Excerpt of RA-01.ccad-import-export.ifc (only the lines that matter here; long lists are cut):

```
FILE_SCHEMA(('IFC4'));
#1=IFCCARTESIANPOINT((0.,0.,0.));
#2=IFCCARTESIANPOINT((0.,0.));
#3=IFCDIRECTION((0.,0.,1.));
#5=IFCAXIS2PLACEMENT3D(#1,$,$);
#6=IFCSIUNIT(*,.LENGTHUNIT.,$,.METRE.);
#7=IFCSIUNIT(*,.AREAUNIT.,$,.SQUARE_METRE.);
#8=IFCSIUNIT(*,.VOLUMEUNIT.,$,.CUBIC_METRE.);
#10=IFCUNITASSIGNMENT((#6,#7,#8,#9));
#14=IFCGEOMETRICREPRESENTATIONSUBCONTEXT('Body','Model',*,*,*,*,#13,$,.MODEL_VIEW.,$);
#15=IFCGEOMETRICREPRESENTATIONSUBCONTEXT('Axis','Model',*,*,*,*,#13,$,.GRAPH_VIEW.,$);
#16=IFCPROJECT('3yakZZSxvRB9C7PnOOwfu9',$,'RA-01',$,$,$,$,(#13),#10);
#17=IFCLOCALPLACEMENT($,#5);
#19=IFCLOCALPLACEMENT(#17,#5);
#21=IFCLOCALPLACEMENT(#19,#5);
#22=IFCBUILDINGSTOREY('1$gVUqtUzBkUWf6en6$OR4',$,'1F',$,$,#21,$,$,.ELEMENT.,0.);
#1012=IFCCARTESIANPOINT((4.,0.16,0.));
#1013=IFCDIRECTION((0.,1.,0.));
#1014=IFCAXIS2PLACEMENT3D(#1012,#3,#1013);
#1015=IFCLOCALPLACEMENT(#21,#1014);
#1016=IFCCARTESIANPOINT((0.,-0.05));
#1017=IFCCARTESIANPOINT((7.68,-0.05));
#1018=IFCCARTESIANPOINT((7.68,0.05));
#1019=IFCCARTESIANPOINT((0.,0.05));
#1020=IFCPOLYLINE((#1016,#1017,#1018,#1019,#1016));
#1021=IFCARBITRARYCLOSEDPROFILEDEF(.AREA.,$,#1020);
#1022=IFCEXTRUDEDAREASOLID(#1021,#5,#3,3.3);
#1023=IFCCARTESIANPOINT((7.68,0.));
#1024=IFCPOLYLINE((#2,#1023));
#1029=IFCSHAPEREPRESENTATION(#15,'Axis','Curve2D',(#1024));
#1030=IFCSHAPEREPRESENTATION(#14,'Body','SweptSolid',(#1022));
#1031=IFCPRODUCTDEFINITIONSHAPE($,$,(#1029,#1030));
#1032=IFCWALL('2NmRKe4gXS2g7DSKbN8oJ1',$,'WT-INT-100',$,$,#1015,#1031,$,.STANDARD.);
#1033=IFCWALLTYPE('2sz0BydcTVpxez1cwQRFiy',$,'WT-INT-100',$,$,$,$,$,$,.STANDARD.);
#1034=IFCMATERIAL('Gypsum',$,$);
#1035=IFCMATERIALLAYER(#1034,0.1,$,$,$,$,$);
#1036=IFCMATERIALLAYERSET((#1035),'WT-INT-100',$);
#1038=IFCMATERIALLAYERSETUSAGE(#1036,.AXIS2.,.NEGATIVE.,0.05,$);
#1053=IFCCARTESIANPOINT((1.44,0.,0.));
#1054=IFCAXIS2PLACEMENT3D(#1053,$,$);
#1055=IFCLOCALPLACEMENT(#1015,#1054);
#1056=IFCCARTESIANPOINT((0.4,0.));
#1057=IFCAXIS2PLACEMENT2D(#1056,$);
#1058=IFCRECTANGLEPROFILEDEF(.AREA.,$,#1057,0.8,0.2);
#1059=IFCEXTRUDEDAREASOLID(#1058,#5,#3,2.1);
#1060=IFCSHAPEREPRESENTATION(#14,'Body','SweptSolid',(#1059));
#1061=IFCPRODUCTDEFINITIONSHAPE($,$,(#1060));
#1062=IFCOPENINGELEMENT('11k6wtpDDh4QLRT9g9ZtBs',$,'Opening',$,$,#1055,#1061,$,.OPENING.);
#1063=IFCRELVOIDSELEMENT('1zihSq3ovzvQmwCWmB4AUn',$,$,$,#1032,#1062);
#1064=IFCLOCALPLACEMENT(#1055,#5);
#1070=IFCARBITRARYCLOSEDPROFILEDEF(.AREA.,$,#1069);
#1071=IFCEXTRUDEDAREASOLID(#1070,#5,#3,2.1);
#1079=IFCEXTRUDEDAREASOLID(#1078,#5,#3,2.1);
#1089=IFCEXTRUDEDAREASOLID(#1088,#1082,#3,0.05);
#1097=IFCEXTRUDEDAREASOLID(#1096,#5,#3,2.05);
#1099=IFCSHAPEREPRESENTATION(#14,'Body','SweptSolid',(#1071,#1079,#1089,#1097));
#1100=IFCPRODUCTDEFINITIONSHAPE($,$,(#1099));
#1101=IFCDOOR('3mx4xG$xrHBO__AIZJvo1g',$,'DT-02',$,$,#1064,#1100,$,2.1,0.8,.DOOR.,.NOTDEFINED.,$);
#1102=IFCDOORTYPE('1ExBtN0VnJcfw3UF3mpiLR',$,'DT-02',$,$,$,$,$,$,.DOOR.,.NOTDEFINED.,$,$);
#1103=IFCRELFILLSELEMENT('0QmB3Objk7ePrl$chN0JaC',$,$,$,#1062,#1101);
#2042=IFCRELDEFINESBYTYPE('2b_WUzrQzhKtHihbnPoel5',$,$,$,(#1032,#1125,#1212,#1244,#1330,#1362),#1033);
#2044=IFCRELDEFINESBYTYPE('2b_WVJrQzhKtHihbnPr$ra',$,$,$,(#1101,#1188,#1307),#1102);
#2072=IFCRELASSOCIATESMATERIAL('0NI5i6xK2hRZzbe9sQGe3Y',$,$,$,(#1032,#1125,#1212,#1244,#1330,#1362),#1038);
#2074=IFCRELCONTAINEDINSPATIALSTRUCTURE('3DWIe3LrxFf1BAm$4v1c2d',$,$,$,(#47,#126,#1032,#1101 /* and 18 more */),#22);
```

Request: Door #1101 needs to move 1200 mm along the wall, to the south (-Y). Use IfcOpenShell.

```python
import ifcopenshell
import ifcopenshell.api.geometry
import ifcopenshell.util.placement
import ifcopenshell.util.unit

model = ifcopenshell.open("RA-01.ccad-import-export.ifc")
unit_scale = ifcopenshell.util.unit.calculate_unit_scale(model)

door = model.by_id(1101)
opening = door.FillsVoids[0].RelatingOpeningElement
wall = opening.VoidsElements[0].RelatingBuildingElement

wall_matrix = ifcopenshell.util.placement.get_local_placement(wall.ObjectPlacement)
shift = wall_matrix[:3, 0] * -1.2 / unit_scale
before = ifcopenshell.util.placement.get_local_placement(door.ObjectPlacement)[:3, 3].copy()

# The door is placed relative to its opening, so it follows when the opening moves.
matrix = ifcopenshell.util.placement.get_local_placement(opening.ObjectPlacement)
matrix[:3, 3] += shift
ifcopenshell.api.geometry.edit_object_placement(
    model, product=opening, matrix=matrix, is_si=False, should_transform_children=True
)

after = ifcopenshell.util.placement.get_local_placement(door.ObjectPlacement)[:3, 3]
print("door moved by", (after - before).round(3) + 0.0)

model.write("RA-01.ccad-import-export_rev.ifc")
```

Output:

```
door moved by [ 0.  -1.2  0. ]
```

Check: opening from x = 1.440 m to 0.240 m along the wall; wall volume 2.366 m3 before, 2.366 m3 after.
